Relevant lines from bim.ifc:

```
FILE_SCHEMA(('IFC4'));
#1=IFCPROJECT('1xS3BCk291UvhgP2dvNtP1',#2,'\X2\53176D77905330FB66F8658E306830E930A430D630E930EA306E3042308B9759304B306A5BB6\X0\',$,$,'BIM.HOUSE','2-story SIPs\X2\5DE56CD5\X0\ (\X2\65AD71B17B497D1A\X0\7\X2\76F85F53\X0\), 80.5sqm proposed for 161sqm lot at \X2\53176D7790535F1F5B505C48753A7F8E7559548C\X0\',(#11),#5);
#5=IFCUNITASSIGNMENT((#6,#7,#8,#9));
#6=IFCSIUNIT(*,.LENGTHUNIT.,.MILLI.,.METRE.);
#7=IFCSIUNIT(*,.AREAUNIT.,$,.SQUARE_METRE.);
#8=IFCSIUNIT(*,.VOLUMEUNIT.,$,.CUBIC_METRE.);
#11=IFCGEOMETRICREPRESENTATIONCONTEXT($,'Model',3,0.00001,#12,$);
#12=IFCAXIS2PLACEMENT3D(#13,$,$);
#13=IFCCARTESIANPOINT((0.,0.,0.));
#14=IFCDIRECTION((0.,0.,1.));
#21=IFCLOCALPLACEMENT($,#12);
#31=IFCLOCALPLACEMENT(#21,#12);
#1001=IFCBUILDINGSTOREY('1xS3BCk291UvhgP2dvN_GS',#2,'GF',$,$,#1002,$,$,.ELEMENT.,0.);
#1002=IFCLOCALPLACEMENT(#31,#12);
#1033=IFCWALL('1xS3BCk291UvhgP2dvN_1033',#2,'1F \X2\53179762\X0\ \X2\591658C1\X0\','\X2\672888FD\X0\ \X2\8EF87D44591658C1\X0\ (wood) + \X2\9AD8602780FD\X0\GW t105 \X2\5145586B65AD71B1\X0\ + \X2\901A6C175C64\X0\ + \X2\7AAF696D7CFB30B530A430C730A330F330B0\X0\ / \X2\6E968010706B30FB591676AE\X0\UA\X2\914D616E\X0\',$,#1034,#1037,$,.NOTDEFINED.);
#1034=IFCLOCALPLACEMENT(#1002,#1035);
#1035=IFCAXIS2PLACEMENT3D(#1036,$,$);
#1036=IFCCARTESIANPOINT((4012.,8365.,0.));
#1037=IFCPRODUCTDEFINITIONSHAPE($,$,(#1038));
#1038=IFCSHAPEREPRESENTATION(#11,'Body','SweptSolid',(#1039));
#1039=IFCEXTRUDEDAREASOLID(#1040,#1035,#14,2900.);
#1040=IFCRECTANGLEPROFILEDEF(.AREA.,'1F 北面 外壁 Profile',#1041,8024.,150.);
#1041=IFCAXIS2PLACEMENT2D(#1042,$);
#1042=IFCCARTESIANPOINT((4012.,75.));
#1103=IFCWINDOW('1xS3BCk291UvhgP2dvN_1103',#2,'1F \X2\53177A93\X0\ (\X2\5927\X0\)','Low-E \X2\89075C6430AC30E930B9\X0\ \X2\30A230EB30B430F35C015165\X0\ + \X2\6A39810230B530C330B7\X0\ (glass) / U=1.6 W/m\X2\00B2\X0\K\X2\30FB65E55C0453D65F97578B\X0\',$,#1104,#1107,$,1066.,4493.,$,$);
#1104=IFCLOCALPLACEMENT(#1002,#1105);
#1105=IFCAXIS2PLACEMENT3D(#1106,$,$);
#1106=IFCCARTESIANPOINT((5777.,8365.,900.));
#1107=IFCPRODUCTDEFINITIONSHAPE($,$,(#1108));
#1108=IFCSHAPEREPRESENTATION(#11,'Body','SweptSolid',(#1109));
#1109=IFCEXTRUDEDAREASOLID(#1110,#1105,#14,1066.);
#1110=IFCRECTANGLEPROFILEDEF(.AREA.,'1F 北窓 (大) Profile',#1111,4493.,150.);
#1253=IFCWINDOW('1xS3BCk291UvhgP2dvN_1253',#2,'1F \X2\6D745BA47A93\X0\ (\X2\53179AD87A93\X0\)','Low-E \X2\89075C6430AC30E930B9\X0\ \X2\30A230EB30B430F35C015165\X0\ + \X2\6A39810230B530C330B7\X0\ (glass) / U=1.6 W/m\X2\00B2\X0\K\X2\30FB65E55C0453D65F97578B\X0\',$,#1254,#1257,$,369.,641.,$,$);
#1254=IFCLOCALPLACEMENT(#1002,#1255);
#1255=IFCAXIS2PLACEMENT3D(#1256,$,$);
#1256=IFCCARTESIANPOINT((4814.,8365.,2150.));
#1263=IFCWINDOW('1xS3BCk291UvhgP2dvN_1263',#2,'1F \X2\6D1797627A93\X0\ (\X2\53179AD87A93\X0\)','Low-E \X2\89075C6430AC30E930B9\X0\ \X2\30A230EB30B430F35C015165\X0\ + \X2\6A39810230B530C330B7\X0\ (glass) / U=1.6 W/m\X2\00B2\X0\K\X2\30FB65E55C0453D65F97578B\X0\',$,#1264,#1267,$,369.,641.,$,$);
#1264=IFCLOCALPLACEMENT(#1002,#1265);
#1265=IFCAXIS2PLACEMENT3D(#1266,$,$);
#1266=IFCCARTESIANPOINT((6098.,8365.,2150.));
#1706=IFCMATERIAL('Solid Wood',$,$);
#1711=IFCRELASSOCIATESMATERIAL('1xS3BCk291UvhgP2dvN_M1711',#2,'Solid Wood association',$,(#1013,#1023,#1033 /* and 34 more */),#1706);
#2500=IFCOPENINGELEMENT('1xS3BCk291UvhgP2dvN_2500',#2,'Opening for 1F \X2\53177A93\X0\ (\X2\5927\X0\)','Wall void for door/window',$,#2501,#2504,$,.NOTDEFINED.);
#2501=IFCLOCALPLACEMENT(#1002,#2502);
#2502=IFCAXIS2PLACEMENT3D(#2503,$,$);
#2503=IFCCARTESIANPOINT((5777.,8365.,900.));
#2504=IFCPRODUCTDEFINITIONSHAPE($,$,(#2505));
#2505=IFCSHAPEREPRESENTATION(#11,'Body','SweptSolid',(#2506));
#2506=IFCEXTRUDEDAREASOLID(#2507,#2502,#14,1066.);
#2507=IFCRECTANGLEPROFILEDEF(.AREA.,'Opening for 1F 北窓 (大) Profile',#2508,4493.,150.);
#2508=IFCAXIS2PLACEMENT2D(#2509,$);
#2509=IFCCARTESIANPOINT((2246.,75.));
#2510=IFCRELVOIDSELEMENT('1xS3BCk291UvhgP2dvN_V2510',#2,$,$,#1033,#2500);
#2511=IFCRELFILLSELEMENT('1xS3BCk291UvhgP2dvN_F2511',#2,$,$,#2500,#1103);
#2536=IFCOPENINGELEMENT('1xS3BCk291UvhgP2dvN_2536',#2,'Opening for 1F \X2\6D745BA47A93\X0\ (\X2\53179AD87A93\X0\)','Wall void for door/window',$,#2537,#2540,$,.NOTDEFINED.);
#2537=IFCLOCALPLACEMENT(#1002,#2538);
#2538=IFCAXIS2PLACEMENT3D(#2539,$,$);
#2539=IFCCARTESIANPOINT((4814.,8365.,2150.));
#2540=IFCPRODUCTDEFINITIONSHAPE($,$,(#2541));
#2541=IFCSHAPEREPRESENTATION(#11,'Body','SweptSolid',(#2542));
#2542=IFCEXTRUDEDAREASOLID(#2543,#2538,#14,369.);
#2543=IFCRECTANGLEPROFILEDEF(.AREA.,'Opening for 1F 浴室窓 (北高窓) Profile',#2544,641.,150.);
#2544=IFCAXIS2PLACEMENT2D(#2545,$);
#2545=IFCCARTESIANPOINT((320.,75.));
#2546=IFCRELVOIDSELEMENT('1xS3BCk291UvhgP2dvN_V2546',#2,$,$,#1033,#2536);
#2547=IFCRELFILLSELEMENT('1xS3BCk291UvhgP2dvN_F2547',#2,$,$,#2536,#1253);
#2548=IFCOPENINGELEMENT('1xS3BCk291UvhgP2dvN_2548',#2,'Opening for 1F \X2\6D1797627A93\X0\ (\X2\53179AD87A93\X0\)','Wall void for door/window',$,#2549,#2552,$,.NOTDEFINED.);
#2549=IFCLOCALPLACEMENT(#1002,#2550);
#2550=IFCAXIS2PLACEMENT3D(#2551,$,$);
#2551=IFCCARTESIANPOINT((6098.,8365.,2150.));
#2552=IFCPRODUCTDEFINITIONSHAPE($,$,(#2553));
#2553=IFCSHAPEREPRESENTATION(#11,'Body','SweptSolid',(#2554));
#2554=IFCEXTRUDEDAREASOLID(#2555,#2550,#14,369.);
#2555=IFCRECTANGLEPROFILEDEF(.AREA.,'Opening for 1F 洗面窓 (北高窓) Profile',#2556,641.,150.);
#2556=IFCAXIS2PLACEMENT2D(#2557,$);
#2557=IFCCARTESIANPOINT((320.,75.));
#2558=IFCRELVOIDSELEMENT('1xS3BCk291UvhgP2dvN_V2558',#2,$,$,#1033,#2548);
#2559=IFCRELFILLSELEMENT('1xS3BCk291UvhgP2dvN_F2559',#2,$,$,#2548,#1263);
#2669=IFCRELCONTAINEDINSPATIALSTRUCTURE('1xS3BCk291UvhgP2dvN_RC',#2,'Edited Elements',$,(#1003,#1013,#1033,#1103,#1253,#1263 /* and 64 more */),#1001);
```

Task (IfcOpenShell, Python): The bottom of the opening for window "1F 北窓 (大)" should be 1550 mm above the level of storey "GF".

```python
import numpy as np
import ifcopenshell
import ifcopenshell.api.geometry
import ifcopenshell.geom
import ifcopenshell.util.element
import ifcopenshell.util.placement
import ifcopenshell.util.shape
import ifcopenshell.util.unit

model = ifcopenshell.open("bim.ifc")
unit_scale = ifcopenshell.util.unit.calculate_unit_scale(model)

window = model.by_guid("1xS3BCk291UvhgP2dvN_1103")
opening = window.FillsVoids[0].RelatingOpeningElement
storey = ifcopenshell.util.element.get_container(window, ifc_class="IfcBuildingStorey")
level = ifcopenshell.util.placement.get_local_placement(storey.ObjectPlacement)[2, 3]

# The opening's origin need not be at the sill, so measure its lowest point.
shape = ifcopenshell.geom.create_shape(ifcopenshell.geom.settings(), opening)
bottom = ifcopenshell.util.shape.get_shape_bottom_elevation(shape, shape.geometry) / unit_scale
dz = level + 1550.0 - bottom

shift = np.array([0.0, 0.0, dz])
# The window is not placed relative to its opening, so move both.
for product in (opening, window):
    matrix = ifcopenshell.util.placement.get_local_placement(product.ObjectPlacement)
    matrix[:3, 3] += shift
    ifcopenshell.api.geometry.edit_object_placement(model, product=product, matrix=matrix, is_si=False)

print(f"moved by {dz * unit_scale:+.3f} m")

model.write("bim-out.ifc")
```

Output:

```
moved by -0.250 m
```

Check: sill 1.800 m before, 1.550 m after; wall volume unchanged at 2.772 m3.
